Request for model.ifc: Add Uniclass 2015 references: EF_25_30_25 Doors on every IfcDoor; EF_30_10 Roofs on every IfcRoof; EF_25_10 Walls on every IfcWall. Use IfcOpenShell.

First a look at what the model holds.

```python
import ifcopenshell

model = ifcopenshell.open("model.ifc")
print(model.schema)
print("classifications:", [c.Name for c in model.by_type("IfcClassification")])
for ifc_class in ("IfcDoor", "IfcRoof", "IfcStair", "IfcWall", "IfcWindow"):
    print(ifc_class, len(model.by_type(ifc_class)))
```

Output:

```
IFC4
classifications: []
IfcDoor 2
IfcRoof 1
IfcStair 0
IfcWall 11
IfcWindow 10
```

```python
import ifcopenshell
import ifcopenshell.api.classification

model = ifcopenshell.open("model.ifc")

system = ifcopenshell.api.classification.add_classification(model, classification="Uniclass 2015")

codes = {
    "IfcDoor": ("EF_25_30_25", "Doors"),
    "IfcRoof": ("EF_30_10", "Roofs"),
    "IfcWall": ("EF_25_10", "Walls"),
}
for ifc_class, (code, name) in codes.items():
    products = model.by_type(ifc_class)
    ifcopenshell.api.classification.add_reference(
        model, products=products, classification=system, identification=code, name=name
    )
    print(code, len(products))

model.write("model_rev.ifc")
```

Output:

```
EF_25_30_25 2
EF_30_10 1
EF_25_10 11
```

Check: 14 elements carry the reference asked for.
